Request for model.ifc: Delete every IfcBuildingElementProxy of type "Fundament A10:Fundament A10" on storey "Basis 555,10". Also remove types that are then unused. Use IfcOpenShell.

First a look at what the model holds.

```python
import ifcopenshell
import ifcopenshell.util.element

model = ifcopenshell.open("model.ifc")
print(model.schema)
storey = next(s for s in model.by_type("IfcBuildingStorey") if s.Name == "Basis 555,10")
proxies = [e for e in ifcopenshell.util.element.get_decomposition(storey) if e.is_a("IfcBuildingElementProxy")]
seen = {}
for e in proxies:
    element_type = ifcopenshell.util.element.get_type(e)
    name = element_type.Name if element_type not in (None, e) else None
    seen[name] = seen.get(name, 0) + 1
for name, count in sorted(seen.items(), key=str):
    print(count, "x", name)
```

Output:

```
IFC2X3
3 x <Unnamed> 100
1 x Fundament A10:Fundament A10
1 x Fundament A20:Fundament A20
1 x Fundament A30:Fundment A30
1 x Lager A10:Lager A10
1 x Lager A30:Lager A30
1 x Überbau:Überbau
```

```python
import ifcopenshell
import ifcopenshell.api.root
import ifcopenshell.util.element

model = ifcopenshell.open("model.ifc")

storey = next(s for s in model.by_type("IfcBuildingStorey") if s.Name == "Basis 555,10")
proxies = [e for e in ifcopenshell.util.element.get_decomposition(storey) if e.is_a("IfcBuildingElementProxy")]
targets = [e for e in proxies if (t := ifcopenshell.util.element.get_type(e)) not in (None, e) and t.Name == "Fundament A10:Fundament A10"]
types = {ifcopenshell.util.element.get_type(e) for e in targets} - {None, *targets}

for e in targets:
    ifcopenshell.api.root.remove_product(model, product=e)
print(len(targets), "removed")

unused = [t for t in types if not ifcopenshell.util.element.get_types(t)]
for t in unused:
    ifcopenshell.api.root.remove_product(model, product=t)
print(len(unused), "unused types removed")

model.write("model_rev.ifc")
```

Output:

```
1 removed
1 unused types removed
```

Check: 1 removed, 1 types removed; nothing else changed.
